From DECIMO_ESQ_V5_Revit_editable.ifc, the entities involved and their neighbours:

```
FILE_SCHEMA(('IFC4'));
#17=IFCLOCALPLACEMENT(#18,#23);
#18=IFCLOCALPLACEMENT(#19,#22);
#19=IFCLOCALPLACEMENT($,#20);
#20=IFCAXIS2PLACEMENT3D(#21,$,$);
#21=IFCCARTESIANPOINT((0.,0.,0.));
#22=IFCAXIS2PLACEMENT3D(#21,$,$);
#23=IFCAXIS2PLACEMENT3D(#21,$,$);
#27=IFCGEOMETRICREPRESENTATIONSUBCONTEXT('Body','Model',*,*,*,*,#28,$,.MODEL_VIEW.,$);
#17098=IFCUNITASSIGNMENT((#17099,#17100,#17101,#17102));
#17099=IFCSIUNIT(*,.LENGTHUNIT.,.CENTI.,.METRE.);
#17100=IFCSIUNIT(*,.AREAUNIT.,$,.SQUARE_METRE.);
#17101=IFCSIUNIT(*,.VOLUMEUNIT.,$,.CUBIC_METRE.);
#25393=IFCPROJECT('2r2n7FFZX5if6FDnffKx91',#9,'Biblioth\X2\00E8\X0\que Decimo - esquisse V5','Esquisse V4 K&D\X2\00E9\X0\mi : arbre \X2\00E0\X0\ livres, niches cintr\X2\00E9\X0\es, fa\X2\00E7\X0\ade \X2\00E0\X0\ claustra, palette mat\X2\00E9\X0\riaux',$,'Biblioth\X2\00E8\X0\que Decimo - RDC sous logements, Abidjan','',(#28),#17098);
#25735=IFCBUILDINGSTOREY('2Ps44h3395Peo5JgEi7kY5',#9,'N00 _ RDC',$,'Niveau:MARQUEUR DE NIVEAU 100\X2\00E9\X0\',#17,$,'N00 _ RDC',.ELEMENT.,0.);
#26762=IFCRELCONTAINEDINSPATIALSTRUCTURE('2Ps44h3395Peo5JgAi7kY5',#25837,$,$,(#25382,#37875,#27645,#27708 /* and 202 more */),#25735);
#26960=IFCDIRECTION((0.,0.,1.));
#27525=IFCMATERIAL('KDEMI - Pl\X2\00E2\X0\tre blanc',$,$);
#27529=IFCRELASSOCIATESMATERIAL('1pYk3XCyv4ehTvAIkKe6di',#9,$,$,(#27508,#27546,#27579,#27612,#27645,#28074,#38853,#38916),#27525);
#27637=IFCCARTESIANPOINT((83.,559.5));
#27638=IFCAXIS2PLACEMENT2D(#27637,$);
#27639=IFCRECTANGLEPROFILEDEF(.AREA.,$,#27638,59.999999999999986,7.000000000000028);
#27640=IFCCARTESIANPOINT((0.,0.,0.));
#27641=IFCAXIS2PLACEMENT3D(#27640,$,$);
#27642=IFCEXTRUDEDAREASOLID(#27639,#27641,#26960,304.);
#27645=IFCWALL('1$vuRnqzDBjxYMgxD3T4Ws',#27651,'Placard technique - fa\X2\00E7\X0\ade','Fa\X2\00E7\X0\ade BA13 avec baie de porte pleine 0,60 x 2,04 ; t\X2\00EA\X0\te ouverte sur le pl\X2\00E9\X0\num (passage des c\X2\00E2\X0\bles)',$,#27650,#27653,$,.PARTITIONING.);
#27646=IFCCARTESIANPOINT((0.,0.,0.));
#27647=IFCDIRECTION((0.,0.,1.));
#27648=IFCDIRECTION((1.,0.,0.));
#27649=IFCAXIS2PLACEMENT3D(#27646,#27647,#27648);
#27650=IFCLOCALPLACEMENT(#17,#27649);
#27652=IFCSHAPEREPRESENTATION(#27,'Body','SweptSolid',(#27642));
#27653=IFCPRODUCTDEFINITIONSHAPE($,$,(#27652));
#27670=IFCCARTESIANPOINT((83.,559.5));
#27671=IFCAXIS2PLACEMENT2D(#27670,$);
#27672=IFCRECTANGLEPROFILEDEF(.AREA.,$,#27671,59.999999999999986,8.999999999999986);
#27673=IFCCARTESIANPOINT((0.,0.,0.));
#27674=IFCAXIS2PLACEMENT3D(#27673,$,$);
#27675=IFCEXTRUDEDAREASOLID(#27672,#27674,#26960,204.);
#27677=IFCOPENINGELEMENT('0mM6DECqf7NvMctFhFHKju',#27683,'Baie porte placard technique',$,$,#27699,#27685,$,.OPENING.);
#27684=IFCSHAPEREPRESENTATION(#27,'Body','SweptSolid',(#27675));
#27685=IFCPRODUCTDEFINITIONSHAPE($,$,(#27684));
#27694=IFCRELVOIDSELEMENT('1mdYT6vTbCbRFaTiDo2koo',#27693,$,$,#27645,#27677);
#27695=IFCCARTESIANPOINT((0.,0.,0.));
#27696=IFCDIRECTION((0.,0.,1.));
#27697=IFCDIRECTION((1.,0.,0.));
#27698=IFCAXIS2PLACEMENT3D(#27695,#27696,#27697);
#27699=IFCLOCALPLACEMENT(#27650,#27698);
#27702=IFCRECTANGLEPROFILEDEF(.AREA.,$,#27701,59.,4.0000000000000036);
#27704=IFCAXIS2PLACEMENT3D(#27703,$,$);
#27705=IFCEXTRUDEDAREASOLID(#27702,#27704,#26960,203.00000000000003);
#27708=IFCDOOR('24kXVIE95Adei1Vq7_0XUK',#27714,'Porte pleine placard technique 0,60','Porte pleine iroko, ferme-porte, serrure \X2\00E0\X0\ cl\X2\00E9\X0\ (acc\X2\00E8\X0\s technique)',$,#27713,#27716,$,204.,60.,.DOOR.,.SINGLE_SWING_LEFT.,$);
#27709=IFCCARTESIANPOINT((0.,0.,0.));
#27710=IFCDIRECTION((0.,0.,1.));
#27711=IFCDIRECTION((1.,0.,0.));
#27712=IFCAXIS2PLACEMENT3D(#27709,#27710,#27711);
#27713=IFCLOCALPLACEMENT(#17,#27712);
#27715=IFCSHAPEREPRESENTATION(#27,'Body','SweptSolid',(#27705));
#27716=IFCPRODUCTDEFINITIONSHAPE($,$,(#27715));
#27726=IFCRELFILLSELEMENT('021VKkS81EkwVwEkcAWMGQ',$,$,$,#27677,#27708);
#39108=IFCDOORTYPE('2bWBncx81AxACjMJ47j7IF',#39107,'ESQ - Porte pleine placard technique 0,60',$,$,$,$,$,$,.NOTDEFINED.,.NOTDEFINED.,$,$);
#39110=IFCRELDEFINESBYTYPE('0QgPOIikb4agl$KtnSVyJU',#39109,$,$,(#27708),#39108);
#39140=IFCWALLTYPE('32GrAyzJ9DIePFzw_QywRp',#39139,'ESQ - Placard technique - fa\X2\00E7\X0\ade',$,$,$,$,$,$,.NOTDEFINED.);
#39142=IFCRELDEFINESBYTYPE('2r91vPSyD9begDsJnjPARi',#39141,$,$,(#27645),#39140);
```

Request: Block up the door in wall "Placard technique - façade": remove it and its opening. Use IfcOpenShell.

```python
import ifcopenshell
import ifcopenshell.api.feature
import ifcopenshell.api.root
import ifcopenshell.geom
import ifcopenshell.util.shape

model = ifcopenshell.open("DECIMO_ESQ_V5_Revit_editable.ifc")
settings = ifcopenshell.geom.settings()


def volume(element):
    """Net volume in cubic metres, openings subtracted."""
    shape = ifcopenshell.geom.create_shape(settings, element)
    return ifcopenshell.util.shape.get_volume(shape.geometry)


door = model.by_guid("24kXVIE95Adei1Vq7_0XUK")
opening = door.FillsVoids[0].RelatingOpeningElement
wall = opening.VoidsElements[0].RelatingBuildingElement
before = volume(wall)

ifcopenshell.api.root.remove_product(model, product=door)
ifcopenshell.api.feature.remove_feature(model, feature=opening)

after = volume(wall)

print(f"wall volume {before:.3f} -> {after:.3f} m3")

model.write("DECIMO_ESQ_V5_Revit_editable_updated.ifc")
```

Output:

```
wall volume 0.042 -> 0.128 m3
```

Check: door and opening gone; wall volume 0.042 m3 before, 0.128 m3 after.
